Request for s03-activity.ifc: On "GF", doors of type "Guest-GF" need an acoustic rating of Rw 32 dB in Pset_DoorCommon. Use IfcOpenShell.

First a look at what the model holds.

```python
import ifcopenshell
import ifcopenshell.util.element

model = ifcopenshell.open("s03-activity.ifc")
print(model.schema)
storey = next(s for s in model.by_type("IfcBuildingStorey") if s.Name == "GF")
doors = [e for e in ifcopenshell.util.element.get_decomposition(storey) if e.is_a("IfcDoor")]
seen = {}
for e in doors:
    element_type = ifcopenshell.util.element.get_type(e)
    key = (element_type.Name if element_type != e and element_type else None, ifcopenshell.util.element.get_pset(e, "Pset_DoorCommon", "AcousticRating"))
    seen[key] = seen.get(key, 0) + 1
for (name, value), count in sorted(seen.items(), key=str):
    print(count, "x", name, "|", value)
```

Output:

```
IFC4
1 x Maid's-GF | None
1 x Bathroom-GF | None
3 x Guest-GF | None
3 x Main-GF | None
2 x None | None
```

```python
import ifcopenshell
import ifcopenshell.api.pset
import ifcopenshell.util.element

model = ifcopenshell.open("s03-activity.ifc")

storey = next(s for s in model.by_type("IfcBuildingStorey") if s.Name == "GF")
doors = [e for e in ifcopenshell.util.element.get_decomposition(storey) if e.is_a("IfcDoor")]

count = 0
for e in doors:
    element_type = ifcopenshell.util.element.get_type(e)
    if element_type in (None, e) or element_type.Name != "Guest-GF":
        continue
    # add_pset returns the element's existing set when there is one.
    pset = ifcopenshell.api.pset.add_pset(model, product=e, name="Pset_DoorCommon")
    ifcopenshell.api.pset.edit_pset(model, pset=pset, properties={"AcousticRating": "Rw 32 dB"})
    count += 1

print(count, "doors updated")

model.write("s03-activity_v2.ifc")
```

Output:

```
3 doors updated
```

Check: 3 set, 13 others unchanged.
